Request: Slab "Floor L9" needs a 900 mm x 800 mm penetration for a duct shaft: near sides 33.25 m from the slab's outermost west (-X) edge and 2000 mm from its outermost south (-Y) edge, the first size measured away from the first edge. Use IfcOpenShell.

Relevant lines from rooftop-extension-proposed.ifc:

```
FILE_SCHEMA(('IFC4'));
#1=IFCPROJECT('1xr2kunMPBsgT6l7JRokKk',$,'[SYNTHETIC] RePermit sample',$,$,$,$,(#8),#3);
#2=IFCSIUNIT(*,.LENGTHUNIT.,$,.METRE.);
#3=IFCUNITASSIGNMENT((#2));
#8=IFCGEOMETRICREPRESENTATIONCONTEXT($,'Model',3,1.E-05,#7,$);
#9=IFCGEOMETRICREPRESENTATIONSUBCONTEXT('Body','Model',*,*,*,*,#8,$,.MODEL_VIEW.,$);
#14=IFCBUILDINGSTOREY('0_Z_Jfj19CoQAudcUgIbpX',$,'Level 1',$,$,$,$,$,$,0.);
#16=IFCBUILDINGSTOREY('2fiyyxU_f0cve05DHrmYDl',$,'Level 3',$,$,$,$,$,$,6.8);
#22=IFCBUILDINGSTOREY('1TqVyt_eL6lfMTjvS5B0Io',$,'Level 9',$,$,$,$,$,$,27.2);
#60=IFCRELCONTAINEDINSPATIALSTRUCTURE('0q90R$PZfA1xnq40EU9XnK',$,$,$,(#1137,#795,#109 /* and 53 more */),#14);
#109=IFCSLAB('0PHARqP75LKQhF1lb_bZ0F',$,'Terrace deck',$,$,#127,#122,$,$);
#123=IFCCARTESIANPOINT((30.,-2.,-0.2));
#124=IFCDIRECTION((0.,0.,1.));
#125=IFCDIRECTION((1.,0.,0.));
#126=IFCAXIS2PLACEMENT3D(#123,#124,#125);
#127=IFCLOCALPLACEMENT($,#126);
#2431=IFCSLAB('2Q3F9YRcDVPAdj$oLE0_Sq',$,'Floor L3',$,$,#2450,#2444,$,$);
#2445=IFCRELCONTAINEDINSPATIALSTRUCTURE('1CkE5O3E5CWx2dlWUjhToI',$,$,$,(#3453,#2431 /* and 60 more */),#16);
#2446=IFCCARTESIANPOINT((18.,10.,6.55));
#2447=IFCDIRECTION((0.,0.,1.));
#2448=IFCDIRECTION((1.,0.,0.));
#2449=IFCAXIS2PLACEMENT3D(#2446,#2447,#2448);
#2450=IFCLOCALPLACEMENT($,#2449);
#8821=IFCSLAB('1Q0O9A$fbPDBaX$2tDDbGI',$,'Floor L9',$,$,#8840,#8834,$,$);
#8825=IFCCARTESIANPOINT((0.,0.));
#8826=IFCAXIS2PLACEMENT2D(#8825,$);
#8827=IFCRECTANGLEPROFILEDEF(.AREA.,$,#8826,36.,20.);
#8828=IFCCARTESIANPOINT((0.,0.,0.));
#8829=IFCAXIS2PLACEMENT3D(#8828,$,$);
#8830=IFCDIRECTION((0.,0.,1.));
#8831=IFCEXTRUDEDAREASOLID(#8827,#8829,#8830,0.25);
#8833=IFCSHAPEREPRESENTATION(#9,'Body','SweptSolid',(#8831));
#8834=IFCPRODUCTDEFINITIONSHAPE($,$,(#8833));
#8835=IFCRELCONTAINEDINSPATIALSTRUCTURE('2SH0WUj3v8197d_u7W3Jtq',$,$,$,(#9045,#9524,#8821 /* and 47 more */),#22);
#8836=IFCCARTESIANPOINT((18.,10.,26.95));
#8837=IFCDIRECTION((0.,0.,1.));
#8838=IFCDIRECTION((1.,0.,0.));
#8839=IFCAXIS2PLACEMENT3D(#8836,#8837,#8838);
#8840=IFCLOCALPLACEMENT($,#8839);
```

```python
import numpy as np
import ifcopenshell
import ifcopenshell.api.feature
import ifcopenshell.api.geometry
import ifcopenshell.api.root
import ifcopenshell.geom
import ifcopenshell.util.placement
import ifcopenshell.util.representation
import ifcopenshell.util.shape
import ifcopenshell.util.unit

model = ifcopenshell.open("rooftop-extension-proposed.ifc")
unit_scale = ifcopenshell.util.unit.calculate_unit_scale(model)
settings = ifcopenshell.geom.settings()


def volume(element):
    """Net volume in cubic metres, openings subtracted."""
    shape = ifcopenshell.geom.create_shape(settings, element)
    return ifcopenshell.util.shape.get_volume(shape.geometry)


slab = model.by_guid("1Q0O9A$fbPDBaX$2tDDbGI")
before = volume(slab)

# Extent in the slab's own axes, in metres. The edges named are its -X and -Y sides.
slab_shape = ifcopenshell.geom.create_shape(settings, slab)
vertices = ifcopenshell.util.shape.get_vertices(slab_shape.geometry)
x_min, y_min, bottom = vertices.min(axis=0)
top = vertices[:, 2].max()

opening = ifcopenshell.api.root.create_entity(model, ifc_class="IfcOpeningElement", name="Duct shaft opening", predefined_type="OPENING")
context = ifcopenshell.util.representation.get_context(model, "Model", "Body", "MODEL_VIEW")
width, depth = 0.9, 0.8
outline = [(0.0, 0.0), (width, 0.0), (width, depth), (0.0, depth), (0.0, 0.0)]
# Overshoot both faces by 50 mm so the cut is clean.
shape = ifcopenshell.api.geometry.add_slab_representation(
    model, context=context, depth=top - bottom + 0.1, polyline=outline
)
ifcopenshell.api.geometry.assign_representation(model, product=opening, representation=shape)

matrix = ifcopenshell.util.placement.get_local_placement(slab.ObjectPlacement)
matrix[:, 3] = matrix @ np.append(np.array([x_min + 33.25, y_min + 2, bottom - 0.05]) / unit_scale, 1.0)
ifcopenshell.api.geometry.edit_object_placement(model, product=opening, matrix=matrix, is_si=False)
ifcopenshell.api.feature.add_feature(model, feature=opening, element=slab)

after = volume(slab)

print(f"slab volume {before:.3f} -> {after:.3f} m3")

model.write("rooftop-extension-proposed_v2.ifc")
```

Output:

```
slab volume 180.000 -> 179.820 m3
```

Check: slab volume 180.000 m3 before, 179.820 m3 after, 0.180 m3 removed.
